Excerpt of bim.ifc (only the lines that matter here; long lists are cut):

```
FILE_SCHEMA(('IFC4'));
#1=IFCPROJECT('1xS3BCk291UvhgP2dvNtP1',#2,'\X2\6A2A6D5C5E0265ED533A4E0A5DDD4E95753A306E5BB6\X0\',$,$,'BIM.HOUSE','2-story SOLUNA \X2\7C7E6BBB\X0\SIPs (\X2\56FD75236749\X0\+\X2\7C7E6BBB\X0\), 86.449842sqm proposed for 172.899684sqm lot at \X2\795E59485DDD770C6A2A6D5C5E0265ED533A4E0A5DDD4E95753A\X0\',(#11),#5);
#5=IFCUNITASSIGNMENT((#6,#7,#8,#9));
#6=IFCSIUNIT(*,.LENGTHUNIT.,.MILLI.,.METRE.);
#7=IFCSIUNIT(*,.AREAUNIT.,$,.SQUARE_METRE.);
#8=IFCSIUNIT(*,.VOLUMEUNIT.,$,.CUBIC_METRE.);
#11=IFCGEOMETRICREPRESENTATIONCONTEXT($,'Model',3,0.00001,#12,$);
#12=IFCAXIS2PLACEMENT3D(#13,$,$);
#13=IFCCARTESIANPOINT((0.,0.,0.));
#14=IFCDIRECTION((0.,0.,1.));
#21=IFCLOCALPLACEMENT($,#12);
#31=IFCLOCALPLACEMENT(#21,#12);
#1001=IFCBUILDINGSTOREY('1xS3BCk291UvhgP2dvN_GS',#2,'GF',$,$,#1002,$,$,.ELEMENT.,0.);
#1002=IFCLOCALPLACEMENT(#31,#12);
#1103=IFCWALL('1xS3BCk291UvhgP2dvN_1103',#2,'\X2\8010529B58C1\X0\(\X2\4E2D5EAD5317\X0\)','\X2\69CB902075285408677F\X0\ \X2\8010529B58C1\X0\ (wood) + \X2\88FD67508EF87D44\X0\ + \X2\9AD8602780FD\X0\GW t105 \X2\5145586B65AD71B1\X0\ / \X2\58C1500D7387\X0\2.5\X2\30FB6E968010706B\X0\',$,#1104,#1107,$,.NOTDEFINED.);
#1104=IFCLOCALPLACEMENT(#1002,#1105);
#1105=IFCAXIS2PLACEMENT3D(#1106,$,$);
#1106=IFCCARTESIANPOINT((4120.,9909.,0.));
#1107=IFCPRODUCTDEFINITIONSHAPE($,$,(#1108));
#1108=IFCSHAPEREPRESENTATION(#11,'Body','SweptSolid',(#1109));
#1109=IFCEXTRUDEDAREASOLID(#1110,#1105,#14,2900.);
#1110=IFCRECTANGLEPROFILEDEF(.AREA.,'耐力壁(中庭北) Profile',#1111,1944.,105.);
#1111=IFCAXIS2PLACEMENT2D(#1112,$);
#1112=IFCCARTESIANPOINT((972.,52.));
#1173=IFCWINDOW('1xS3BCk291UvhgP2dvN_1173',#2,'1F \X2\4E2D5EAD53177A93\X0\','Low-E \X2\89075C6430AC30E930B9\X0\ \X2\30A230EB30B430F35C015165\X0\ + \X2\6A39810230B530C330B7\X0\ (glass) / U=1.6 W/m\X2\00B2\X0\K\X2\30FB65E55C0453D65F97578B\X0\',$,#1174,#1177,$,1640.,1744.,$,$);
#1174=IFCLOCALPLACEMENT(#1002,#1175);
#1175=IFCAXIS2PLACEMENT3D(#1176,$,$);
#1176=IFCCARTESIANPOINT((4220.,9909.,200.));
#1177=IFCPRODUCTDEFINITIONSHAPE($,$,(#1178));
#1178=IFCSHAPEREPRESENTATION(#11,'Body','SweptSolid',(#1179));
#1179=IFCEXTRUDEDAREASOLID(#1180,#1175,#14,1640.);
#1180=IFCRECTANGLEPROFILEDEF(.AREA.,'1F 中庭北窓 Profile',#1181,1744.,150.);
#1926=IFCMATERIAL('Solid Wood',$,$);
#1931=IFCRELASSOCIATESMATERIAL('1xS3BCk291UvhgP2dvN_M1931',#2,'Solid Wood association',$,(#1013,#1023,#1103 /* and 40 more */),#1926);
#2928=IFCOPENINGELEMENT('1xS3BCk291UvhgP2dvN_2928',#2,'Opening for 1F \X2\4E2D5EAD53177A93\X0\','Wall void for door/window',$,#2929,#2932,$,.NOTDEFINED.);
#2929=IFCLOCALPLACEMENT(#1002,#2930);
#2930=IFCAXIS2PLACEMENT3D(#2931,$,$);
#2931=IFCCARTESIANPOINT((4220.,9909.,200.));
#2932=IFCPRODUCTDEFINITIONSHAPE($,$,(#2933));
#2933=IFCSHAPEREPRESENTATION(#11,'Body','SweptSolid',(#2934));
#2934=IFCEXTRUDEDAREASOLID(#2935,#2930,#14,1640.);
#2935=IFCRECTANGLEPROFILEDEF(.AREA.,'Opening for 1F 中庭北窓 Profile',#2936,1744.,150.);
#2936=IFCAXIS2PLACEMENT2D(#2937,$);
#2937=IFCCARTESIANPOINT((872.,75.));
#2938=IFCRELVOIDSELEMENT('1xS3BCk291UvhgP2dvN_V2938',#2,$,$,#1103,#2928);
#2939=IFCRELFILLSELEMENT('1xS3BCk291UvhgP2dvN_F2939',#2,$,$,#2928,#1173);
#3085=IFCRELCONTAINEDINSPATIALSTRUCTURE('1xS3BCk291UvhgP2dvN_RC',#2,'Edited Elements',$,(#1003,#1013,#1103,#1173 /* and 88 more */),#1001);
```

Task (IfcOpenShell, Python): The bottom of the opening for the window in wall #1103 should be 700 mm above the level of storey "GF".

```python
import numpy as np
import ifcopenshell
import ifcopenshell.api.geometry
import ifcopenshell.geom
import ifcopenshell.util.element
import ifcopenshell.util.placement
import ifcopenshell.util.shape
import ifcopenshell.util.unit

model = ifcopenshell.open("bim.ifc")
unit_scale = ifcopenshell.util.unit.calculate_unit_scale(model)

window = model.by_id(1173)
opening = window.FillsVoids[0].RelatingOpeningElement
storey = ifcopenshell.util.element.get_container(window, ifc_class="IfcBuildingStorey")
level = ifcopenshell.util.placement.get_local_placement(storey.ObjectPlacement)[2, 3]

# The opening's origin need not be at the sill, so measure its lowest point.
shape = ifcopenshell.geom.create_shape(ifcopenshell.geom.settings(), opening)
bottom = ifcopenshell.util.shape.get_shape_bottom_elevation(shape, shape.geometry) / unit_scale
dz = level + 700.0 - bottom

shift = np.array([0.0, 0.0, dz])
# The window is not placed relative to its opening, so move both.
for product in (opening, window):
    matrix = ifcopenshell.util.placement.get_local_placement(product.ObjectPlacement)
    matrix[:3, 3] += shift
    ifcopenshell.api.geometry.edit_object_placement(model, product=product, matrix=matrix, is_si=False)

print(f"moved by {dz * unit_scale:+.3f} m")

model.write("bim_v2.ifc")
```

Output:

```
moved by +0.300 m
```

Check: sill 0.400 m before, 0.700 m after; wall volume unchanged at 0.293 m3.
